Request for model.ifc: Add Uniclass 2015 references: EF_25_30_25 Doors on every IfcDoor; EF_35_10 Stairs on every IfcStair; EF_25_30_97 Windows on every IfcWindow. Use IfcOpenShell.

First a look at what the model holds.

```python
import ifcopenshell

model = ifcopenshell.open("model.ifc")
print(model.schema)
print("classifications:", [c.Name for c in model.by_type("IfcClassification")])
for ifc_class in ("IfcDoor", "IfcRoof", "IfcStair", "IfcWall", "IfcWindow"):
    print(ifc_class, len(model.by_type(ifc_class)))
```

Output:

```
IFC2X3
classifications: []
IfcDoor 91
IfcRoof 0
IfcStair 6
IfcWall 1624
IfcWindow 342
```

```python
import ifcopenshell
import ifcopenshell.api.classification

model = ifcopenshell.open("model.ifc")

# IFC2X3 requires Source and Edition and has no link from the project to the system.
system = model.create_entity("IfcClassification", Source="NBS", Edition="2015", Name="Uniclass 2015")

codes = {
    "IfcDoor": ("EF_25_30_25", "Doors"),
    "IfcStair": ("EF_35_10", "Stairs"),
    "IfcWindow": ("EF_25_30_97", "Windows"),
}
for ifc_class, (code, name) in codes.items():
    products = model.by_type(ifc_class)
    ifcopenshell.api.classification.add_reference(
        model, products=products, classification=system, identification=code, name=name
    )
    print(code, len(products))

model.write("model_rev.ifc")
```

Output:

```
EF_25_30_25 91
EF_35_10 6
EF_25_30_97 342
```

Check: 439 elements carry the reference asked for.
